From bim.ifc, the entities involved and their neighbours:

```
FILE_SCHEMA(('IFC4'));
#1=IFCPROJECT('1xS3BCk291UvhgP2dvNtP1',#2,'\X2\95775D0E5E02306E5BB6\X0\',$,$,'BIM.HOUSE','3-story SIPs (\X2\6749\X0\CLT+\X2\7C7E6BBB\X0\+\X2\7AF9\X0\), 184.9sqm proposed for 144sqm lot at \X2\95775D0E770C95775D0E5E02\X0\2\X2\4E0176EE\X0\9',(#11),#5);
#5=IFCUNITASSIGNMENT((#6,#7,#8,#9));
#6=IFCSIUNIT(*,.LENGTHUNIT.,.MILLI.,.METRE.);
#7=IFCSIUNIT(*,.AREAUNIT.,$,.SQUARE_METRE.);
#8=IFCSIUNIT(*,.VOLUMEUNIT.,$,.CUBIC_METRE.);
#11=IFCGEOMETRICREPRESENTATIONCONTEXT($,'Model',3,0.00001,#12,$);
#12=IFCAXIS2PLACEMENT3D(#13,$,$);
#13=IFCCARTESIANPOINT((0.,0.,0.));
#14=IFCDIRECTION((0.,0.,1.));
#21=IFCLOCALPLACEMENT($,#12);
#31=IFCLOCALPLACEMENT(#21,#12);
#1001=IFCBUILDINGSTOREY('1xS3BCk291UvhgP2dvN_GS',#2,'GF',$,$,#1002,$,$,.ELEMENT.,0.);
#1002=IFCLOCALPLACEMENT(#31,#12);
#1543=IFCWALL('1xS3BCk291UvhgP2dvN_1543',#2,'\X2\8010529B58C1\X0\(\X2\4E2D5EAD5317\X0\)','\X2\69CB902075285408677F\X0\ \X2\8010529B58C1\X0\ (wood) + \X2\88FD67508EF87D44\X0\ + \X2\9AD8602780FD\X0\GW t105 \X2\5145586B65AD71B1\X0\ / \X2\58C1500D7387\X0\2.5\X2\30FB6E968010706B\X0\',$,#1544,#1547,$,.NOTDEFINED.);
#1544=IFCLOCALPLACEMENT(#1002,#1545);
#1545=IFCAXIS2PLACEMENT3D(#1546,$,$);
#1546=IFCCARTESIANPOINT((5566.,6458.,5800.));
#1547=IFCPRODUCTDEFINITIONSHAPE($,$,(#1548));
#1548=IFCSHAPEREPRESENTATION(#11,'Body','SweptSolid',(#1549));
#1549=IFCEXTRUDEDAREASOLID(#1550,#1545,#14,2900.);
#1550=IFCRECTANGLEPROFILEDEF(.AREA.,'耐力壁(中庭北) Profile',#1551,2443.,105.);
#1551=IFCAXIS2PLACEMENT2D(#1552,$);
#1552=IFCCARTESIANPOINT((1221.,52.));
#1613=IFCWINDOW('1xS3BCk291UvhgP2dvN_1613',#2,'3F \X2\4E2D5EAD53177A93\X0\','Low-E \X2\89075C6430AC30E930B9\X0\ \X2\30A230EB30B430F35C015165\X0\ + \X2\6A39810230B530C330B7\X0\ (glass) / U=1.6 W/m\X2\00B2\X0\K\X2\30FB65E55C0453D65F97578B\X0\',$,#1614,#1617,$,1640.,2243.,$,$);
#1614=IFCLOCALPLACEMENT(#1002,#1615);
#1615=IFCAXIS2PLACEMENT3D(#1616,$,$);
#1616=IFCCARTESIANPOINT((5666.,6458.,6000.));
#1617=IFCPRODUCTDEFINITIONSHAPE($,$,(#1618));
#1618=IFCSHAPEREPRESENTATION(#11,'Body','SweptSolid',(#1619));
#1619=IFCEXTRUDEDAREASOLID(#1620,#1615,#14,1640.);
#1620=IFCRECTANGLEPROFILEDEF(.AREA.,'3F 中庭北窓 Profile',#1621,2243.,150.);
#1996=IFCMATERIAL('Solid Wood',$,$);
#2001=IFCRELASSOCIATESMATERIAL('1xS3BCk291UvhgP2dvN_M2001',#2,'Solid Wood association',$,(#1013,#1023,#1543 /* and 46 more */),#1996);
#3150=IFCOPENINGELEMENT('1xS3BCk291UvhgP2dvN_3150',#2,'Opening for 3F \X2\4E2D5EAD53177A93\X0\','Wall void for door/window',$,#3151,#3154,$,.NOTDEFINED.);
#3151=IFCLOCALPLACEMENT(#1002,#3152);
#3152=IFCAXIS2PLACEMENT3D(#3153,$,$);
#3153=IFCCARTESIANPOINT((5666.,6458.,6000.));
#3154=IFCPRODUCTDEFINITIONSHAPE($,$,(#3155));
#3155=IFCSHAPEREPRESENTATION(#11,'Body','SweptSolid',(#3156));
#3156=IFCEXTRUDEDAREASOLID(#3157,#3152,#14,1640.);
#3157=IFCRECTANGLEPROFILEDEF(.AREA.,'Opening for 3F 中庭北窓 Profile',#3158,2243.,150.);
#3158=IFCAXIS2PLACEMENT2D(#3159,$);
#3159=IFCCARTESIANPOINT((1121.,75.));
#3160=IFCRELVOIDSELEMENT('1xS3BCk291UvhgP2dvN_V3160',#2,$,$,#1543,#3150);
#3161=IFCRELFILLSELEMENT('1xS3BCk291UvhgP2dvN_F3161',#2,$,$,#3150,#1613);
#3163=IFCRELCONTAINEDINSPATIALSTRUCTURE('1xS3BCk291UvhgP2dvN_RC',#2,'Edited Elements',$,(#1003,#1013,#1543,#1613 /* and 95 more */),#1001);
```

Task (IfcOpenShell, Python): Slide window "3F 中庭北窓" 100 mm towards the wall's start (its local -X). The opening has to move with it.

```python
import ifcopenshell
import ifcopenshell.api.geometry
import ifcopenshell.util.placement

model = ifcopenshell.open("bim.ifc")

window = model.by_guid("1xS3BCk291UvhgP2dvN_1613")
opening = window.FillsVoids[0].RelatingOpeningElement
wall = opening.VoidsElements[0].RelatingBuildingElement

wall_matrix = ifcopenshell.util.placement.get_local_placement(wall.ObjectPlacement)
shift = wall_matrix[:3, 0] * -100.0
before = ifcopenshell.util.placement.get_local_placement(window.ObjectPlacement)[:3, 3].copy()

# The window is not placed relative to its opening, so move both.
for product in (opening, window):
    matrix = ifcopenshell.util.placement.get_local_placement(product.ObjectPlacement)
    matrix[:3, 3] += shift
    ifcopenshell.api.geometry.edit_object_placement(model, product=product, matrix=matrix, is_si=False)

after = ifcopenshell.util.placement.get_local_placement(window.ObjectPlacement)[:3, 3]
print("window moved by", (after - before).round(3) + 0.0)

model.write("bim-out.ifc")
```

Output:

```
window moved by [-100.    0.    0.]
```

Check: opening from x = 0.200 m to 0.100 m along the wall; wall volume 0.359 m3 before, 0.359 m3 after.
